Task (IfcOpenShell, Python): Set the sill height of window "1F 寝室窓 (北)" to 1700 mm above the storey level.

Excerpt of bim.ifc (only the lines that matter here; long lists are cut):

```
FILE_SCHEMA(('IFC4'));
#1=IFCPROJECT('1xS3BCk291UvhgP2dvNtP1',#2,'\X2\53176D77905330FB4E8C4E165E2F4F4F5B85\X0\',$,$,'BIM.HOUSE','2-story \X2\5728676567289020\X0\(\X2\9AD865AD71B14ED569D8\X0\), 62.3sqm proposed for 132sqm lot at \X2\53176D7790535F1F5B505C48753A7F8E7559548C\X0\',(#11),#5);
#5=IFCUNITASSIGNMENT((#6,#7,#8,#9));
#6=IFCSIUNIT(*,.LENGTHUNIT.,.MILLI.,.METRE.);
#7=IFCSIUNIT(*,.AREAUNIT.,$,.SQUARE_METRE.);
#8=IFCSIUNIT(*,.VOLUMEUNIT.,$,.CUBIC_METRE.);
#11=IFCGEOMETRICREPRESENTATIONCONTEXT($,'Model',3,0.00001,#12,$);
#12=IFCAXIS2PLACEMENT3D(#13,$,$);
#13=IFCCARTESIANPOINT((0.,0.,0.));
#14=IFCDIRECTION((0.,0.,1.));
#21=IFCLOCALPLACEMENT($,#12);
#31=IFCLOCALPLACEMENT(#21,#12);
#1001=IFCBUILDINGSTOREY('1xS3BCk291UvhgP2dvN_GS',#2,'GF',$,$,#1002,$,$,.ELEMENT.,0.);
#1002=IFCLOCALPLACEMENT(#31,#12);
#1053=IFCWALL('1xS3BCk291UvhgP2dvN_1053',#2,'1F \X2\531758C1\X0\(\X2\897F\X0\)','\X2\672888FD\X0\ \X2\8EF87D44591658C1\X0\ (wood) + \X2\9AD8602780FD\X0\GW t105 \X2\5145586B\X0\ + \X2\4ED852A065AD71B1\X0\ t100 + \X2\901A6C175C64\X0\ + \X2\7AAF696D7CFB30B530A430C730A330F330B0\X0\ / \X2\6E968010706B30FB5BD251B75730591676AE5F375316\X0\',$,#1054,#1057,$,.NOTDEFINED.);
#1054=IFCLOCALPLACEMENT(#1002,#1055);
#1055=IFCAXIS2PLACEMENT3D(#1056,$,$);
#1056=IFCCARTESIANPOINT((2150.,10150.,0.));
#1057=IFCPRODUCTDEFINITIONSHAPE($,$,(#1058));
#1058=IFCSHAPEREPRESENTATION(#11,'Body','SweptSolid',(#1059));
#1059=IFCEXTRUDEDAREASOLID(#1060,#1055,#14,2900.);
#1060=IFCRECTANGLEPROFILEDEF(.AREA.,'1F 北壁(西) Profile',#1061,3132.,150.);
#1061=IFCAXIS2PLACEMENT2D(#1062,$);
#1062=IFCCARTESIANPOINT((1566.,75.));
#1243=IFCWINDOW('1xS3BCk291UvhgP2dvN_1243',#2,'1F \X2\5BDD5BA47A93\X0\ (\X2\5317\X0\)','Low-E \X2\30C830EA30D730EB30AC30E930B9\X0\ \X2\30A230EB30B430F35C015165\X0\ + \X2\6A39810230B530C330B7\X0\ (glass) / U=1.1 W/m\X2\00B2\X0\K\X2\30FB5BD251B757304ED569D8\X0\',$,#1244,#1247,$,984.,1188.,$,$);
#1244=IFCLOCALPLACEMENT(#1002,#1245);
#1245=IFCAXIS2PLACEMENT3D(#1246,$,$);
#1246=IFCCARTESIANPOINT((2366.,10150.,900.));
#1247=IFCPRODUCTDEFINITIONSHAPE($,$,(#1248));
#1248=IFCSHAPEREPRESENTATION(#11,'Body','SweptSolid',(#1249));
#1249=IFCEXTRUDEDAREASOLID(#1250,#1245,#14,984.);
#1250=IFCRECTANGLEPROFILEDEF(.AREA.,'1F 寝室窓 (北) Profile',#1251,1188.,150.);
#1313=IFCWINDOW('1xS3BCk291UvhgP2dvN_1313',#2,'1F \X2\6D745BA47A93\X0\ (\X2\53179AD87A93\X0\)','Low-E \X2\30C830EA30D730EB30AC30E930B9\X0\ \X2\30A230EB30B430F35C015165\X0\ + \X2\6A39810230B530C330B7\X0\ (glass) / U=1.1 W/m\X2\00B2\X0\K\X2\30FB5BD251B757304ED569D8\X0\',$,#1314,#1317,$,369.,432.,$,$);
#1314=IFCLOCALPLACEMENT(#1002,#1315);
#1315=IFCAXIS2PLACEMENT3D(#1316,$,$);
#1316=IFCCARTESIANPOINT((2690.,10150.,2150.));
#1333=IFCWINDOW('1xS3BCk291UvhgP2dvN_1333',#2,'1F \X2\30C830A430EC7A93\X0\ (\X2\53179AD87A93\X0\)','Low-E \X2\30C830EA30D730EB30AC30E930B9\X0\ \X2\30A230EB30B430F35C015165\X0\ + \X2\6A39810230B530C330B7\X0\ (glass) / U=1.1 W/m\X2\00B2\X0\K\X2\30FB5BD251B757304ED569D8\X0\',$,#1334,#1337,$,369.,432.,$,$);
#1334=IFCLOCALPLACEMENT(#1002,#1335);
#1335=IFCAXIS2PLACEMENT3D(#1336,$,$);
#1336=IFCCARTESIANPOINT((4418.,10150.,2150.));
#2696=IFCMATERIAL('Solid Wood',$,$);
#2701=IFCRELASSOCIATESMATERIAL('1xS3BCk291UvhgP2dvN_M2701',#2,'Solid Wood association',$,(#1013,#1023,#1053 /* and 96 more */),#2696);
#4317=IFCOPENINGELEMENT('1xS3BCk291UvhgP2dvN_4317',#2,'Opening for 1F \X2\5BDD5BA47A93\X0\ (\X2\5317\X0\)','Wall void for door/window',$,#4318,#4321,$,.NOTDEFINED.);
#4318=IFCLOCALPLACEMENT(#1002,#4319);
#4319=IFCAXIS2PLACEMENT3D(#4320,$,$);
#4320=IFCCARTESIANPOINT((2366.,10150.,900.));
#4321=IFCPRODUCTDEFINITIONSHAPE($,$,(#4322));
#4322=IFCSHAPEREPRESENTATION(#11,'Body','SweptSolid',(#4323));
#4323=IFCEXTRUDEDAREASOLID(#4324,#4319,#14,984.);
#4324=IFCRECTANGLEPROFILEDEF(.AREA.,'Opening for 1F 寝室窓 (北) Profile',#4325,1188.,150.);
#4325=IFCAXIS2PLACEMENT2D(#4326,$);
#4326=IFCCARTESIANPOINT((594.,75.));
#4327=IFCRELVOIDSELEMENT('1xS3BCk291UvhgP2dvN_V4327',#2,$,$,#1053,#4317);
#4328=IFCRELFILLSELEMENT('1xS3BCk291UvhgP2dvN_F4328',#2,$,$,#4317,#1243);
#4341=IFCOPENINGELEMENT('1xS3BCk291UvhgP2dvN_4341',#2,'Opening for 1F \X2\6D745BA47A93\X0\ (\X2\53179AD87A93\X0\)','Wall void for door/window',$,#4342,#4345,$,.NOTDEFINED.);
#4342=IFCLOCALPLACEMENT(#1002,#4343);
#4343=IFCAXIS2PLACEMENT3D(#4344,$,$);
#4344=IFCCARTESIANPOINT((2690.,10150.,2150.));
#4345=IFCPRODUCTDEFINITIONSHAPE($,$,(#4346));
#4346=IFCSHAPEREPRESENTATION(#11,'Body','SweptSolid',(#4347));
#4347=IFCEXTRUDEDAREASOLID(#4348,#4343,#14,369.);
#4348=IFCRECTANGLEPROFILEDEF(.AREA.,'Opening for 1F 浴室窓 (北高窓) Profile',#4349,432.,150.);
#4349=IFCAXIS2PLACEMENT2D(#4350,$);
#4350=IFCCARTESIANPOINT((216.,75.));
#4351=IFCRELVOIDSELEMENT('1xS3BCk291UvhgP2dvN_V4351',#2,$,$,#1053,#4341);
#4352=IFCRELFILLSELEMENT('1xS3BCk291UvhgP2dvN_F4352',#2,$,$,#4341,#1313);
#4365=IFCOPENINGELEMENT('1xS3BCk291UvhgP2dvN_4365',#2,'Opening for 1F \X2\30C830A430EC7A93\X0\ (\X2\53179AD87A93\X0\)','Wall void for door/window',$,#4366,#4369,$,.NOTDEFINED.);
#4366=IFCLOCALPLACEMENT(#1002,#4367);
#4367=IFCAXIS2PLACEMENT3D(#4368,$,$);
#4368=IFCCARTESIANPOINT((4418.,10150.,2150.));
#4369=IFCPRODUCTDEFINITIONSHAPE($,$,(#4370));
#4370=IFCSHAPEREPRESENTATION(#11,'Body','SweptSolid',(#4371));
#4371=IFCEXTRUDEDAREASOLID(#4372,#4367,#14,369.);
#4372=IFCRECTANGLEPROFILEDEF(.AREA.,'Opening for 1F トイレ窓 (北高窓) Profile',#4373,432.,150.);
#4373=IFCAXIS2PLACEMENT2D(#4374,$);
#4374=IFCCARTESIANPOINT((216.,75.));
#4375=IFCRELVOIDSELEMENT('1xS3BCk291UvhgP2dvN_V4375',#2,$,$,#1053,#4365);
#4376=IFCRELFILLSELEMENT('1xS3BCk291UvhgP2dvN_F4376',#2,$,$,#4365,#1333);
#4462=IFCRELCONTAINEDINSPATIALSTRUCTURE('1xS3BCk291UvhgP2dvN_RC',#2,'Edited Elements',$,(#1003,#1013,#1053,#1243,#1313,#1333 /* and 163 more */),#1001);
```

```python
import numpy as np
import ifcopenshell
import ifcopenshell.api.geometry
import ifcopenshell.geom
import ifcopenshell.util.element
import ifcopenshell.util.placement
import ifcopenshell.util.shape
import ifcopenshell.util.unit

model = ifcopenshell.open("bim.ifc")
unit_scale = ifcopenshell.util.unit.calculate_unit_scale(model)

window = model.by_id(1243)
opening = window.FillsVoids[0].RelatingOpeningElement
storey = ifcopenshell.util.element.get_container(window, ifc_class="IfcBuildingStorey")
level = ifcopenshell.util.placement.get_local_placement(storey.ObjectPlacement)[2, 3]

# The opening's origin need not be at the sill, so measure its lowest point.
shape = ifcopenshell.geom.create_shape(ifcopenshell.geom.settings(), opening)
bottom = ifcopenshell.util.shape.get_shape_bottom_elevation(shape, shape.geometry) / unit_scale
dz = level + 1.7 / unit_scale - bottom

shift = np.array([0.0, 0.0, dz])
# The window is not placed relative to its opening, so move both.
for product in (opening, window):
    matrix = ifcopenshell.util.placement.get_local_placement(product.ObjectPlacement)
    matrix[:3, 3] += shift
    ifcopenshell.api.geometry.edit_object_placement(model, product=product, matrix=matrix, is_si=False)

print(f"moved by {dz * unit_scale:+.3f} m")

model.write("bim_v2.ifc")
```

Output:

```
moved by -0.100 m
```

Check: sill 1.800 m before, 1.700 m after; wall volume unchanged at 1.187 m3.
